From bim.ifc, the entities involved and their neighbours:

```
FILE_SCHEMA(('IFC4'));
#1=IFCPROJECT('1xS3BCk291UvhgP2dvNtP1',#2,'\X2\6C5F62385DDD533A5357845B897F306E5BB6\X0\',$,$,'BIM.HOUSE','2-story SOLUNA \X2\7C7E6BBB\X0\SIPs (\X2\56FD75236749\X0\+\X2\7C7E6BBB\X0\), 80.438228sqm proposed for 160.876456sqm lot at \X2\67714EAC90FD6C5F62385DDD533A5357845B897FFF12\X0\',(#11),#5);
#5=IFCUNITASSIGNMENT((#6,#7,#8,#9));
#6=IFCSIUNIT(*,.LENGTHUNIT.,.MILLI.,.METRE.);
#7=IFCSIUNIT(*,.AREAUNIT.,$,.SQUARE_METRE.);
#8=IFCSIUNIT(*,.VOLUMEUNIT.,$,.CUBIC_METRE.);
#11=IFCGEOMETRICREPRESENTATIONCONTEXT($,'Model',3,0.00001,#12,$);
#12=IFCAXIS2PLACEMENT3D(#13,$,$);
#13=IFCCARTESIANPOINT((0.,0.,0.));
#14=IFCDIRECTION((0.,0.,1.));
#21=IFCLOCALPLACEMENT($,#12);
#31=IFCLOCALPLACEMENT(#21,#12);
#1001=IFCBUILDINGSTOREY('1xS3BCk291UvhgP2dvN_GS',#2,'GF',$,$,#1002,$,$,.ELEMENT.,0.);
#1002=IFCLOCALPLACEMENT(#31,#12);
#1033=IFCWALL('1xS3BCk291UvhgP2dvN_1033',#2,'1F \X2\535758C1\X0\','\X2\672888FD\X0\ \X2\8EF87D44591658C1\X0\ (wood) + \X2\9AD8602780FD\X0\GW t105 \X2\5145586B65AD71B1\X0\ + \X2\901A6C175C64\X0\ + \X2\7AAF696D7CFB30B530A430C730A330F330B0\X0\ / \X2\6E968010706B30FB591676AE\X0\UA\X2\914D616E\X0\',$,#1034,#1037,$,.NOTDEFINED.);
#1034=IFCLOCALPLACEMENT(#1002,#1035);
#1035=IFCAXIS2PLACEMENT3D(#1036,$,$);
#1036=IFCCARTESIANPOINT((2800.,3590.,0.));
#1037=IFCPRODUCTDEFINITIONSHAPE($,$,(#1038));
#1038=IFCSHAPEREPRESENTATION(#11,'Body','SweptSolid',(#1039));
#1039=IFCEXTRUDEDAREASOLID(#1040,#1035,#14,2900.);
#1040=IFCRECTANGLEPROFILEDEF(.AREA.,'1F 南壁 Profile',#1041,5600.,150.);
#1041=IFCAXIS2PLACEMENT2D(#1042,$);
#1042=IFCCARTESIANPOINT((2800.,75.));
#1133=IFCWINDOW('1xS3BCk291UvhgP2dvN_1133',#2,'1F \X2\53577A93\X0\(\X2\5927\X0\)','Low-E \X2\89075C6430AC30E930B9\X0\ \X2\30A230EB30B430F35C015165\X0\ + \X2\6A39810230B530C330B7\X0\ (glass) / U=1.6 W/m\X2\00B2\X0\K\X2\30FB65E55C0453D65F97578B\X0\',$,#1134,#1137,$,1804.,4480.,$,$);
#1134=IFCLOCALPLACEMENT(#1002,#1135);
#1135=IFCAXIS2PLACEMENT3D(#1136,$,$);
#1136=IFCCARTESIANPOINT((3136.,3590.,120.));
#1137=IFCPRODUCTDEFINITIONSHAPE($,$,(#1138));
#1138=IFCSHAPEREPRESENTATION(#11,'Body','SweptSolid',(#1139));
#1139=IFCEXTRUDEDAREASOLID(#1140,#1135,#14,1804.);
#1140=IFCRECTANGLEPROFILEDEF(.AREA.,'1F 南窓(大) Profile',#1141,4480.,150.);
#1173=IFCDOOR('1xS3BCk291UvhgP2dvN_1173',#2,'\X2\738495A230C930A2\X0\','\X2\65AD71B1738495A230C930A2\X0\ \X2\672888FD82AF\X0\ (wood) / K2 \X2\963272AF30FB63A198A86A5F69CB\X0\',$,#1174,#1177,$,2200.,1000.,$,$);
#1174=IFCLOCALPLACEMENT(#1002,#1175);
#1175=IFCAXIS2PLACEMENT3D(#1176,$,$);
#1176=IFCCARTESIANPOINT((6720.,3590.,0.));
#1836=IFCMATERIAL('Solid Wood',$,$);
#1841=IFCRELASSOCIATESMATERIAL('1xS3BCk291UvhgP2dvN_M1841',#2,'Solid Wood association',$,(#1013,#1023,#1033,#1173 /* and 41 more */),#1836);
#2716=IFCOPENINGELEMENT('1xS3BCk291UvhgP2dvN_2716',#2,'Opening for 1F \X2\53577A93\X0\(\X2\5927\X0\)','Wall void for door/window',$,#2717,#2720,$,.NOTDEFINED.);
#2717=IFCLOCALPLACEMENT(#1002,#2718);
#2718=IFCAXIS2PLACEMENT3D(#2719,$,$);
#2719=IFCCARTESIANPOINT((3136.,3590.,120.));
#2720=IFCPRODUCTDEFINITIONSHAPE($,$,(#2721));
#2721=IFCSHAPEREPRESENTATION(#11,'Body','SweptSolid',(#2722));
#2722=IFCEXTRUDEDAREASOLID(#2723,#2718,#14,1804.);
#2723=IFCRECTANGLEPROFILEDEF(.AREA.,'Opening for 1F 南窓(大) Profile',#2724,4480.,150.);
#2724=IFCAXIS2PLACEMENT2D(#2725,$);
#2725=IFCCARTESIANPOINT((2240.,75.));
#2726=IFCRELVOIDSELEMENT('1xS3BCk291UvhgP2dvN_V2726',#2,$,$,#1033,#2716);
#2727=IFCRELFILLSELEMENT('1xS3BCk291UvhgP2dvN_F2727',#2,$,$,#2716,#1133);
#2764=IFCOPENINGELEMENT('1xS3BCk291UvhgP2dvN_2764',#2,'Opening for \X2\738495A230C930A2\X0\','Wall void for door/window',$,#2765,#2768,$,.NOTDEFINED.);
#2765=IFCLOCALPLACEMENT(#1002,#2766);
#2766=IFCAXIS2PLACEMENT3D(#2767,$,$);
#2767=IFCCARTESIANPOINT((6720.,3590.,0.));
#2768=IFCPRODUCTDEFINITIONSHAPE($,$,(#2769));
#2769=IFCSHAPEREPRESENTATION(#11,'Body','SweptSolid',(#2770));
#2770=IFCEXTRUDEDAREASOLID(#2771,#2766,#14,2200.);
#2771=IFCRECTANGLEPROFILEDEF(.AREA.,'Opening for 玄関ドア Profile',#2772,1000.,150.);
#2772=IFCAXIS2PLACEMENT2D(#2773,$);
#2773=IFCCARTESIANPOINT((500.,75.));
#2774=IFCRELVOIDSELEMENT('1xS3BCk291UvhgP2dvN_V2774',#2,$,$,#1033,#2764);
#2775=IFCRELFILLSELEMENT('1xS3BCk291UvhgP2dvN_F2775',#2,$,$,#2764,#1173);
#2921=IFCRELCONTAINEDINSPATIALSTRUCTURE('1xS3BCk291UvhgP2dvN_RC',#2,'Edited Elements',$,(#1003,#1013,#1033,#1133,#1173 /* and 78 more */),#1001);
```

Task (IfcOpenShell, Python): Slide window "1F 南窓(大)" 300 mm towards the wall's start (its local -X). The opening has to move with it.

```python
import ifcopenshell
import ifcopenshell.api.geometry
import ifcopenshell.util.placement
import ifcopenshell.util.unit

model = ifcopenshell.open("bim.ifc")
unit_scale = ifcopenshell.util.unit.calculate_unit_scale(model)

window = model.by_guid("1xS3BCk291UvhgP2dvN_1133")
opening = window.FillsVoids[0].RelatingOpeningElement
wall = opening.VoidsElements[0].RelatingBuildingElement

wall_matrix = ifcopenshell.util.placement.get_local_placement(wall.ObjectPlacement)
shift = wall_matrix[:3, 0] * -0.3 / unit_scale
before = ifcopenshell.util.placement.get_local_placement(window.ObjectPlacement)[:3, 3].copy()

# The window is not placed relative to its opening, so move both.
for product in (opening, window):
    matrix = ifcopenshell.util.placement.get_local_placement(product.ObjectPlacement)
    matrix[:3, 3] += shift
    ifcopenshell.api.geometry.edit_object_placement(model, product=product, matrix=matrix, is_si=False)

after = ifcopenshell.util.placement.get_local_placement(window.ObjectPlacement)[:3, 3]
print("window moved by", (after - before).round(3) + 0.0)

model.write("bim_rev.ifc")
```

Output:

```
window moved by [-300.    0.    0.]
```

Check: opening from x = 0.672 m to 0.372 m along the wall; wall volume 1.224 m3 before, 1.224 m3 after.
